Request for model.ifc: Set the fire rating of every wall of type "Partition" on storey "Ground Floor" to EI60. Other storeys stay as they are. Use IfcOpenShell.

First a look at what the model holds.

```python
import ifcopenshell
import ifcopenshell.util.element

model = ifcopenshell.open("model.ifc")
print(model.schema)
storey = next(s for s in model.by_type("IfcBuildingStorey") if s.Name == "Ground Floor")
walls = [e for e in ifcopenshell.util.element.get_decomposition(storey) if e.is_a("IfcWall")]
seen = {}
for e in walls:
    element_type = ifcopenshell.util.element.get_type(e)
    key = (element_type.Name if element_type != e and element_type else None, ifcopenshell.util.element.get_pset(e, "Pset_WallCommon", "FireRating"))
    seen[key] = seen.get(key, 0) + 1
for (name, value), count in sorted(seen.items(), key=str):
    print(count, "x", name, "|", value)
```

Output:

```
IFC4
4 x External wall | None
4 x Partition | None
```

```python
import ifcopenshell
import ifcopenshell.api.pset
import ifcopenshell.util.element

model = ifcopenshell.open("model.ifc")

storey = next(s for s in model.by_type("IfcBuildingStorey") if s.Name == "Ground Floor")
walls = [e for e in ifcopenshell.util.element.get_decomposition(storey) if e.is_a("IfcWall")]

count = 0
for e in walls:
    element_type = ifcopenshell.util.element.get_type(e)
    if element_type in (None, e) or element_type.Name != "Partition":
        continue
    # add_pset returns the element's existing set when there is one.
    pset = ifcopenshell.api.pset.add_pset(model, product=e, name="Pset_WallCommon")
    ifcopenshell.api.pset.edit_pset(model, pset=pset, properties={"FireRating": "EI60"})
    count += 1

print(count, "walls updated")

model.write("model_edited.ifc")
```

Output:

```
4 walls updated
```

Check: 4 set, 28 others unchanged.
